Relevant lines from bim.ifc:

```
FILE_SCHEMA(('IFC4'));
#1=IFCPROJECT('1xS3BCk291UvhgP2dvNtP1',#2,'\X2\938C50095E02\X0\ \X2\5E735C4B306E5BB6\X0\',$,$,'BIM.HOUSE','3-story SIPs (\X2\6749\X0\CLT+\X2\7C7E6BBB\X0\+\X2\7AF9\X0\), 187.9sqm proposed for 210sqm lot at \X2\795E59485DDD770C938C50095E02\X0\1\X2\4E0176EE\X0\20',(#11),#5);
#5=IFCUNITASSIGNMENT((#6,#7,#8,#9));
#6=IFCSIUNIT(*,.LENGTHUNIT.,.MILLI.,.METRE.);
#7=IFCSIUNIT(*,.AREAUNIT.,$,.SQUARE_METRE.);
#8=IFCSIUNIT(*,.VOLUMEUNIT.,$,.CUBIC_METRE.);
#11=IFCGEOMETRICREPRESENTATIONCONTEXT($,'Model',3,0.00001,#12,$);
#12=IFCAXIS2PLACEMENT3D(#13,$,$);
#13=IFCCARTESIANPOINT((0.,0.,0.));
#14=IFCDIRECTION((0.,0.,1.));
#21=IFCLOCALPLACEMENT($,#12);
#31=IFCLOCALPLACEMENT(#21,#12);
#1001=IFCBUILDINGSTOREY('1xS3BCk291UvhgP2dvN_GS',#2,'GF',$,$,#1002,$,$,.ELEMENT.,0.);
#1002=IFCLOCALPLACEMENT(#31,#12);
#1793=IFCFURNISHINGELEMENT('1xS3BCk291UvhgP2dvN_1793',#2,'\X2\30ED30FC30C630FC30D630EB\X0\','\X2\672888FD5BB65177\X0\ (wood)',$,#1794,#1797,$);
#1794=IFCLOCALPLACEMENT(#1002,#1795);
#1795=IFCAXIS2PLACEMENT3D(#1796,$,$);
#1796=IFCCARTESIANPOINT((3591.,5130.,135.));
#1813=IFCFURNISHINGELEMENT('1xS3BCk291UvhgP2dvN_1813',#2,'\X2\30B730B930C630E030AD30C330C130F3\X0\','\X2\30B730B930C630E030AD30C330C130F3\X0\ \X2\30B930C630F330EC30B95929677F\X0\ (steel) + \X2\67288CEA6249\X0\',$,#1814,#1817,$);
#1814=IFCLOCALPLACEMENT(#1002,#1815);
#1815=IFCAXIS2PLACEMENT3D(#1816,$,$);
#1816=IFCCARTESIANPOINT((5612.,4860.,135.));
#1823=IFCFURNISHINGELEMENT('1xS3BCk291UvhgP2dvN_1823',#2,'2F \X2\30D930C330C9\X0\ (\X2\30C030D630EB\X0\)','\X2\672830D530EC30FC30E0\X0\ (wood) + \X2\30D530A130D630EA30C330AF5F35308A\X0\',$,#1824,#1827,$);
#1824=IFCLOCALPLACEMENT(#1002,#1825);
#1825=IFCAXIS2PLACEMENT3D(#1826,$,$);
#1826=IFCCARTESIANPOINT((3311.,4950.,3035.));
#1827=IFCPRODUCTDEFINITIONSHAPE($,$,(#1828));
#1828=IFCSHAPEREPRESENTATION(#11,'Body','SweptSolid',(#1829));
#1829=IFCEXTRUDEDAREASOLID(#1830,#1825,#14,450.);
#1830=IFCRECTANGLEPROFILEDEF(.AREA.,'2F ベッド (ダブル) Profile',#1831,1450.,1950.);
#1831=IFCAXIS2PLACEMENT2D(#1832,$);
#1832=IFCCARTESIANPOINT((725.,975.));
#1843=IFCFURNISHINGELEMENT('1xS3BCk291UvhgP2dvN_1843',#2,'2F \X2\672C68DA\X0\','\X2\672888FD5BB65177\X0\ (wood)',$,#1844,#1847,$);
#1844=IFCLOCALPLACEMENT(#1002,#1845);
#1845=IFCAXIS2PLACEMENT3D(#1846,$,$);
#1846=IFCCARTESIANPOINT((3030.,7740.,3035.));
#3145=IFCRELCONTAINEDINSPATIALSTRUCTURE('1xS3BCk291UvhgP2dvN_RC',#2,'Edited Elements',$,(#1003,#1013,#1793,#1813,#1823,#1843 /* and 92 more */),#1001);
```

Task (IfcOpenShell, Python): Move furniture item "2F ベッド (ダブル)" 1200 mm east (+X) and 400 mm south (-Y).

```python
import ifcopenshell
import ifcopenshell.api.geometry
import ifcopenshell.util.placement

model = ifcopenshell.open("bim.ifc")

item = model.by_guid("1xS3BCk291UvhgP2dvN_1823")
matrix = ifcopenshell.util.placement.get_local_placement(item.ObjectPlacement)
matrix[0, 3] += 1200.0
matrix[1, 3] -= 400.0
ifcopenshell.api.geometry.edit_object_placement(model, product=item, matrix=matrix, is_si=False)

print(ifcopenshell.util.placement.get_local_placement(item.ObjectPlacement).round(3) + 0.0)

model.write("bim-out.ifc")
```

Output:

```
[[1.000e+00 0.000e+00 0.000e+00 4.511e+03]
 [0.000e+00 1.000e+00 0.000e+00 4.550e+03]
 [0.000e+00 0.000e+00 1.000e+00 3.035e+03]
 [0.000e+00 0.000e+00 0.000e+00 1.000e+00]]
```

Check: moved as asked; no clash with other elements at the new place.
